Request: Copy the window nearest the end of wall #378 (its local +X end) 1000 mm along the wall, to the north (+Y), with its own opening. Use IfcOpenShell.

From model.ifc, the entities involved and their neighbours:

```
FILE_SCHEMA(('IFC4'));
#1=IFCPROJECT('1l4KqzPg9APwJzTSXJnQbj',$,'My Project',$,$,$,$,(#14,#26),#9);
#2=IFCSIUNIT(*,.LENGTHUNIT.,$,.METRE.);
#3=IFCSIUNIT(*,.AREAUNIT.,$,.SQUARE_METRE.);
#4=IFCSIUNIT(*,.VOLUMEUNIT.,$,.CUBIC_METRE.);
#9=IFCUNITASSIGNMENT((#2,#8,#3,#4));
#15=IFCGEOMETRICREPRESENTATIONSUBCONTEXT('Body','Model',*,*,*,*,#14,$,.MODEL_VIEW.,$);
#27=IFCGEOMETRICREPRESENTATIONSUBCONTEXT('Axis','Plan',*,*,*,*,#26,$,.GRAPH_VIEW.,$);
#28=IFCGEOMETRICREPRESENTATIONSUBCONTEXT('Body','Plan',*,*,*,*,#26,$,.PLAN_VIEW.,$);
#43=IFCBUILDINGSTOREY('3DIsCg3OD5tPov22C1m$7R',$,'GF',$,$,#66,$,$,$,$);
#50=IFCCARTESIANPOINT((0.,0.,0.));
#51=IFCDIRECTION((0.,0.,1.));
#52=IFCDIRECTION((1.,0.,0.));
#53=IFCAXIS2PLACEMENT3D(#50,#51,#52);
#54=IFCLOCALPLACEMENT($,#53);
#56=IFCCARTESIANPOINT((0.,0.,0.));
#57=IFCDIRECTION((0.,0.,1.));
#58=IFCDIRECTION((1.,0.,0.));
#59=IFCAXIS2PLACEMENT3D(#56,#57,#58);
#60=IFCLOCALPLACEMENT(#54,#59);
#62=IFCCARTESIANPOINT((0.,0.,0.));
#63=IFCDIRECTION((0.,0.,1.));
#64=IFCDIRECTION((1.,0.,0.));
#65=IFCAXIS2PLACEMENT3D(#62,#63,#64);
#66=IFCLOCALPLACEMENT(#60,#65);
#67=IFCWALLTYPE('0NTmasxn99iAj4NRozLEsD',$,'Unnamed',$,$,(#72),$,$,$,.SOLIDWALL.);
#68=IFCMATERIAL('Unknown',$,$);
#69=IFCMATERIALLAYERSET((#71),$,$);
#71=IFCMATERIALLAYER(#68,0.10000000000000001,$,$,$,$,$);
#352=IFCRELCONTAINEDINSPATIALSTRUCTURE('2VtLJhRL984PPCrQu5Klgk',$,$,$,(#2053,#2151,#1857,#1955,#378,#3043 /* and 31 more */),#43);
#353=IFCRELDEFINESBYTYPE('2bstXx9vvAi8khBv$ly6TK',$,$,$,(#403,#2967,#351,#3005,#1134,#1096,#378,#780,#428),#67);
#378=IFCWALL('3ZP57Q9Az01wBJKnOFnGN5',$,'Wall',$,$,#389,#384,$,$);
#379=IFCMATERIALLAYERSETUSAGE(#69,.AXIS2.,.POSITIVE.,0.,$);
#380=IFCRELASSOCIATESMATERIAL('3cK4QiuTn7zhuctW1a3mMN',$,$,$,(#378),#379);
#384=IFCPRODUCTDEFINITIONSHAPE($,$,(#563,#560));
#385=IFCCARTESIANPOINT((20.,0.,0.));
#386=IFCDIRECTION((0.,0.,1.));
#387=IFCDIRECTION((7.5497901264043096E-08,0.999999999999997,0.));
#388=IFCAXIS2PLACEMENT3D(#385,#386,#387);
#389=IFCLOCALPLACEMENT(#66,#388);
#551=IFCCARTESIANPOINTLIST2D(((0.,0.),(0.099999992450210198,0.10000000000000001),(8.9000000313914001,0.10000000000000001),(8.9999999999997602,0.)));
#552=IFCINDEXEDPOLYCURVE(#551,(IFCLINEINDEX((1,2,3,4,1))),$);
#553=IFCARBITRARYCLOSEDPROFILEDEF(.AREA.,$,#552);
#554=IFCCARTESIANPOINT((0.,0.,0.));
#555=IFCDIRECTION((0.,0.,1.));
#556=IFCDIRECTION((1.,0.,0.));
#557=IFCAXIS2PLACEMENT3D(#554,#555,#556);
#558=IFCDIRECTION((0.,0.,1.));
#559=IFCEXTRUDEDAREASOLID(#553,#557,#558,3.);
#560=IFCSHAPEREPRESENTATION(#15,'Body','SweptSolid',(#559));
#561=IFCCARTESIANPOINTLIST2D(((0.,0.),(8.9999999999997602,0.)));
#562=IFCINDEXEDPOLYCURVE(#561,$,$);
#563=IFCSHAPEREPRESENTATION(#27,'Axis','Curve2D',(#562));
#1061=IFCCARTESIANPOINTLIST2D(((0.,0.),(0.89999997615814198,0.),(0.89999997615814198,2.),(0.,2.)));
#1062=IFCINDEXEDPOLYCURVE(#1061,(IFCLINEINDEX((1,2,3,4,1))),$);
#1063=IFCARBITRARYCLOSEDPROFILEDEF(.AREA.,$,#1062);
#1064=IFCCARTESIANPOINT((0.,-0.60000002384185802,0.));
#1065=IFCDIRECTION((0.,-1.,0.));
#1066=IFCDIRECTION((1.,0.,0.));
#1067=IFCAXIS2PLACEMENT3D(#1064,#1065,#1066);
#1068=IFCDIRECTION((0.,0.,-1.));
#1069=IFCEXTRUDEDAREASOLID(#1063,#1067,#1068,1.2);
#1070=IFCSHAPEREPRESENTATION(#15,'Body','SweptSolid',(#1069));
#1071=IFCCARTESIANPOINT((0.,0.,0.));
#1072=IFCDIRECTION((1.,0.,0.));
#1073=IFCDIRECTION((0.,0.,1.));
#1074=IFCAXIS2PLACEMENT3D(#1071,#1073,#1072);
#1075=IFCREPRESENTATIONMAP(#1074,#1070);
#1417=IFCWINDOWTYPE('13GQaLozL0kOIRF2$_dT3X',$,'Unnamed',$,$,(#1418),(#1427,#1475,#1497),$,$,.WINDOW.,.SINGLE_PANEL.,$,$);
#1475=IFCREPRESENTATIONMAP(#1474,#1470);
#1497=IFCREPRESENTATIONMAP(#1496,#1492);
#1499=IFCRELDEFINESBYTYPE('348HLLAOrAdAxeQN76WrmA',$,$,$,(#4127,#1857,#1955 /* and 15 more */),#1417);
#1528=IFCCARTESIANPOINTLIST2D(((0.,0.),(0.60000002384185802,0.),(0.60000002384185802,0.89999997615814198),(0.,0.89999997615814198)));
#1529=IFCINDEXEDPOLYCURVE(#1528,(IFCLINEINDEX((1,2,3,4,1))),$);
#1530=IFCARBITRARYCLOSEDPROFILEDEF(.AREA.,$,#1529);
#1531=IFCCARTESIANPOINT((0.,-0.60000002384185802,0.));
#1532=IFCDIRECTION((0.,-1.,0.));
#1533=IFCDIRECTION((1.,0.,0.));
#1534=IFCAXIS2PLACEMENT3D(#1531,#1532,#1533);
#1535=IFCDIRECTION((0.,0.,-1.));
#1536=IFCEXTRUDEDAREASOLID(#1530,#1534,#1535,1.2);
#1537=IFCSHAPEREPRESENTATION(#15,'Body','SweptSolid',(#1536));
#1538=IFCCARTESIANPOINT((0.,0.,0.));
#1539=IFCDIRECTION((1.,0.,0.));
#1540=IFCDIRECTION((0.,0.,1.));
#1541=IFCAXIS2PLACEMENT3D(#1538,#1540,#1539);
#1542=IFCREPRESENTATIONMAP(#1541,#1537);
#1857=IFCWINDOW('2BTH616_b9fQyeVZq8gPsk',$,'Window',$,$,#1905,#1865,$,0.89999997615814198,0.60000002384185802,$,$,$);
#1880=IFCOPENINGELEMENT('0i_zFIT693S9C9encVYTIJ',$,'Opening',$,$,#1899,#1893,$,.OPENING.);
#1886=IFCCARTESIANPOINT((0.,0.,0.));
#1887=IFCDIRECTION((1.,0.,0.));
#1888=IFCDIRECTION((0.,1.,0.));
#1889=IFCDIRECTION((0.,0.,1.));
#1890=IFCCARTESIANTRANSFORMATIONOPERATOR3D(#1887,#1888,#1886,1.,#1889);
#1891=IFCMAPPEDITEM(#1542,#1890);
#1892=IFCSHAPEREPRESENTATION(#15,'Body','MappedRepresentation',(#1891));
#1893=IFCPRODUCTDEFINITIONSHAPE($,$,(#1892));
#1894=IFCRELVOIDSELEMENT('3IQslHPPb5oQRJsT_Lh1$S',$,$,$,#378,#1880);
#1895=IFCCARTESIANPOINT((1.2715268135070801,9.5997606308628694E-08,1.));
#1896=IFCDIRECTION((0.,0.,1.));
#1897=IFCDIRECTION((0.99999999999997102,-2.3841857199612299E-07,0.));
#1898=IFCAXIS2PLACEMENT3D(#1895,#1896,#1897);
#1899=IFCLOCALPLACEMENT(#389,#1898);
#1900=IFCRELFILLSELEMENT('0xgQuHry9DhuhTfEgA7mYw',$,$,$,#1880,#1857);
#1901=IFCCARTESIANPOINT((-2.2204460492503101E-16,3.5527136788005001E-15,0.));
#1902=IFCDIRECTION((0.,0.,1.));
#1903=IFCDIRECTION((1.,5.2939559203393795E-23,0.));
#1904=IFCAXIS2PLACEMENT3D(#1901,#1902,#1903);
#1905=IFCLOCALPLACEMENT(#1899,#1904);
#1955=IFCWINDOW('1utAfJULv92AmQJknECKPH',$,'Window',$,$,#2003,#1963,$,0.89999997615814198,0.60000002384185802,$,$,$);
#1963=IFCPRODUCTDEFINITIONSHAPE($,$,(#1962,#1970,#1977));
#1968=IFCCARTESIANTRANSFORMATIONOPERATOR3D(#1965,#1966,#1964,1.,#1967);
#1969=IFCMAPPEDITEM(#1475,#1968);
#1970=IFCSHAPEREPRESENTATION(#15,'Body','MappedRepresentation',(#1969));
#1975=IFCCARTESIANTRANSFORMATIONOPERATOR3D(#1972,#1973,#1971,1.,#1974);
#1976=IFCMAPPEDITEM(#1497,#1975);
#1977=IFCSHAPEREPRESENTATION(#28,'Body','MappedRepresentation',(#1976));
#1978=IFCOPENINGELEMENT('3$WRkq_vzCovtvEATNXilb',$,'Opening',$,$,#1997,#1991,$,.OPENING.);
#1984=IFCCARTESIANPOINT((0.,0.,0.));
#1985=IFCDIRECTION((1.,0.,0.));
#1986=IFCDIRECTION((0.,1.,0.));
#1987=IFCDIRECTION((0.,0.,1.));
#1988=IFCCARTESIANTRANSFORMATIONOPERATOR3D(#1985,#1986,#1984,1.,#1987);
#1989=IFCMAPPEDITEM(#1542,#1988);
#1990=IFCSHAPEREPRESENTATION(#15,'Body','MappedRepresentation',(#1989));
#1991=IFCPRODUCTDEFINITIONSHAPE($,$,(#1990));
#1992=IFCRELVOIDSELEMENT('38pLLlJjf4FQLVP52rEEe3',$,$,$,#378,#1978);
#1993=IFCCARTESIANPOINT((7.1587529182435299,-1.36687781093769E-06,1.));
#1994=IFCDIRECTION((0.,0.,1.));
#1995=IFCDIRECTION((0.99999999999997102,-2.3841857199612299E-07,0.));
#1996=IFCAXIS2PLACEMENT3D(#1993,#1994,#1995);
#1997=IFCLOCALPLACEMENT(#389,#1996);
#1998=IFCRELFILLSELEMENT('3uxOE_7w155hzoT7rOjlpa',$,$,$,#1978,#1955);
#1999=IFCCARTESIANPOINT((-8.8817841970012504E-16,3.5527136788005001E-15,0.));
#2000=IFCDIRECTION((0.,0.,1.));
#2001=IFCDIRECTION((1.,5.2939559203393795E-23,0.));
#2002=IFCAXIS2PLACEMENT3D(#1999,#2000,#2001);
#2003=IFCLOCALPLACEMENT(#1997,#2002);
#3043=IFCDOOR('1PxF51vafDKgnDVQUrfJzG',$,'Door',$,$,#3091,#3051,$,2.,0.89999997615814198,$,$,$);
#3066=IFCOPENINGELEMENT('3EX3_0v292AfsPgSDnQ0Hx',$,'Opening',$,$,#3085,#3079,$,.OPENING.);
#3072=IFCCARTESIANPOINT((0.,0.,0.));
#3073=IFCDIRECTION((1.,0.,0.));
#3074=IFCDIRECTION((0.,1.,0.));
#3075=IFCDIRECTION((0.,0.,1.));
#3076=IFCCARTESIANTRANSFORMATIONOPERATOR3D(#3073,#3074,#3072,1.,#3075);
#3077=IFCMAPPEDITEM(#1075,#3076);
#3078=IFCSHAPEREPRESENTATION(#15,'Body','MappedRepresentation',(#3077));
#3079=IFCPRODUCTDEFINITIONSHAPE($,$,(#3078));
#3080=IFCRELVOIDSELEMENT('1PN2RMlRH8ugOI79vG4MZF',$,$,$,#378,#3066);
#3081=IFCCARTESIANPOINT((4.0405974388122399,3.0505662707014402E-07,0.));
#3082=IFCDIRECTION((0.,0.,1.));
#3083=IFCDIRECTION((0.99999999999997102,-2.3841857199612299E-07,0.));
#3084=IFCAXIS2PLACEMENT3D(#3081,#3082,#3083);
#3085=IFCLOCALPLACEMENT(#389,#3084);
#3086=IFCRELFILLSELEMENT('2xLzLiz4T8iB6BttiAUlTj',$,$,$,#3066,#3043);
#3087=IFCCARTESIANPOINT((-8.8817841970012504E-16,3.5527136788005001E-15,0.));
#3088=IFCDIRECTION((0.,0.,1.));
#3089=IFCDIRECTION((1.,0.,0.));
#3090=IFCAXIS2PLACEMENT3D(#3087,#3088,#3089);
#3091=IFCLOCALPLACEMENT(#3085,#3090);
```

```python
import ifcopenshell
import ifcopenshell.api.feature
import ifcopenshell.api.geometry
import ifcopenshell.api.root
import ifcopenshell.geom
import ifcopenshell.util.element
import ifcopenshell.util.placement
import ifcopenshell.util.shape
import ifcopenshell.util.unit

model = ifcopenshell.open("model.ifc")
unit_scale = ifcopenshell.util.unit.calculate_unit_scale(model)
settings = ifcopenshell.geom.settings()


def volume(element):
    """Net volume in cubic metres, openings subtracted."""
    shape = ifcopenshell.geom.create_shape(settings, element)
    return ifcopenshell.util.shape.get_volume(shape.geometry)


window = model.by_guid("1utAfJULv92AmQJknECKPH")
opening = window.FillsVoids[0].RelatingOpeningElement
wall = opening.VoidsElements[0].RelatingBuildingElement
before = volume(wall)
shift = ifcopenshell.util.placement.get_local_placement(wall.ObjectPlacement)[:3, 0] * 1 / unit_scale

# copy_class copies the void relationship, type, container and properties, but no geometry.
new_opening = ifcopenshell.api.root.copy_class(model, product=opening)
new_opening.Representation = ifcopenshell.util.element.copy_deep(
    model, opening.Representation, exclude=["IfcGeometricRepresentationContext", "IfcRepresentationMap"]
)
new_window = ifcopenshell.api.root.copy_class(model, product=window)
new_window.Representation = ifcopenshell.util.element.copy_deep(
    model, window.Representation, exclude=["IfcGeometricRepresentationContext", "IfcRepresentationMap"]
)
ifcopenshell.api.feature.add_filling(model, opening=new_opening, element=new_window)

for old, new in ((opening, new_opening), (window, new_window)):
    matrix = ifcopenshell.util.placement.get_local_placement(old.ObjectPlacement)
    matrix[:3, 3] += shift
    ifcopenshell.api.geometry.edit_object_placement(model, product=new, matrix=matrix, is_si=False)

after = volume(wall)

print(f"wall volume {before:.3f} -> {after:.3f} m3")

model.write("model_updated.ifc")
```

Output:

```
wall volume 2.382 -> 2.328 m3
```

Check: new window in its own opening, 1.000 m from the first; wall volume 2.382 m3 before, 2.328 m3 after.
